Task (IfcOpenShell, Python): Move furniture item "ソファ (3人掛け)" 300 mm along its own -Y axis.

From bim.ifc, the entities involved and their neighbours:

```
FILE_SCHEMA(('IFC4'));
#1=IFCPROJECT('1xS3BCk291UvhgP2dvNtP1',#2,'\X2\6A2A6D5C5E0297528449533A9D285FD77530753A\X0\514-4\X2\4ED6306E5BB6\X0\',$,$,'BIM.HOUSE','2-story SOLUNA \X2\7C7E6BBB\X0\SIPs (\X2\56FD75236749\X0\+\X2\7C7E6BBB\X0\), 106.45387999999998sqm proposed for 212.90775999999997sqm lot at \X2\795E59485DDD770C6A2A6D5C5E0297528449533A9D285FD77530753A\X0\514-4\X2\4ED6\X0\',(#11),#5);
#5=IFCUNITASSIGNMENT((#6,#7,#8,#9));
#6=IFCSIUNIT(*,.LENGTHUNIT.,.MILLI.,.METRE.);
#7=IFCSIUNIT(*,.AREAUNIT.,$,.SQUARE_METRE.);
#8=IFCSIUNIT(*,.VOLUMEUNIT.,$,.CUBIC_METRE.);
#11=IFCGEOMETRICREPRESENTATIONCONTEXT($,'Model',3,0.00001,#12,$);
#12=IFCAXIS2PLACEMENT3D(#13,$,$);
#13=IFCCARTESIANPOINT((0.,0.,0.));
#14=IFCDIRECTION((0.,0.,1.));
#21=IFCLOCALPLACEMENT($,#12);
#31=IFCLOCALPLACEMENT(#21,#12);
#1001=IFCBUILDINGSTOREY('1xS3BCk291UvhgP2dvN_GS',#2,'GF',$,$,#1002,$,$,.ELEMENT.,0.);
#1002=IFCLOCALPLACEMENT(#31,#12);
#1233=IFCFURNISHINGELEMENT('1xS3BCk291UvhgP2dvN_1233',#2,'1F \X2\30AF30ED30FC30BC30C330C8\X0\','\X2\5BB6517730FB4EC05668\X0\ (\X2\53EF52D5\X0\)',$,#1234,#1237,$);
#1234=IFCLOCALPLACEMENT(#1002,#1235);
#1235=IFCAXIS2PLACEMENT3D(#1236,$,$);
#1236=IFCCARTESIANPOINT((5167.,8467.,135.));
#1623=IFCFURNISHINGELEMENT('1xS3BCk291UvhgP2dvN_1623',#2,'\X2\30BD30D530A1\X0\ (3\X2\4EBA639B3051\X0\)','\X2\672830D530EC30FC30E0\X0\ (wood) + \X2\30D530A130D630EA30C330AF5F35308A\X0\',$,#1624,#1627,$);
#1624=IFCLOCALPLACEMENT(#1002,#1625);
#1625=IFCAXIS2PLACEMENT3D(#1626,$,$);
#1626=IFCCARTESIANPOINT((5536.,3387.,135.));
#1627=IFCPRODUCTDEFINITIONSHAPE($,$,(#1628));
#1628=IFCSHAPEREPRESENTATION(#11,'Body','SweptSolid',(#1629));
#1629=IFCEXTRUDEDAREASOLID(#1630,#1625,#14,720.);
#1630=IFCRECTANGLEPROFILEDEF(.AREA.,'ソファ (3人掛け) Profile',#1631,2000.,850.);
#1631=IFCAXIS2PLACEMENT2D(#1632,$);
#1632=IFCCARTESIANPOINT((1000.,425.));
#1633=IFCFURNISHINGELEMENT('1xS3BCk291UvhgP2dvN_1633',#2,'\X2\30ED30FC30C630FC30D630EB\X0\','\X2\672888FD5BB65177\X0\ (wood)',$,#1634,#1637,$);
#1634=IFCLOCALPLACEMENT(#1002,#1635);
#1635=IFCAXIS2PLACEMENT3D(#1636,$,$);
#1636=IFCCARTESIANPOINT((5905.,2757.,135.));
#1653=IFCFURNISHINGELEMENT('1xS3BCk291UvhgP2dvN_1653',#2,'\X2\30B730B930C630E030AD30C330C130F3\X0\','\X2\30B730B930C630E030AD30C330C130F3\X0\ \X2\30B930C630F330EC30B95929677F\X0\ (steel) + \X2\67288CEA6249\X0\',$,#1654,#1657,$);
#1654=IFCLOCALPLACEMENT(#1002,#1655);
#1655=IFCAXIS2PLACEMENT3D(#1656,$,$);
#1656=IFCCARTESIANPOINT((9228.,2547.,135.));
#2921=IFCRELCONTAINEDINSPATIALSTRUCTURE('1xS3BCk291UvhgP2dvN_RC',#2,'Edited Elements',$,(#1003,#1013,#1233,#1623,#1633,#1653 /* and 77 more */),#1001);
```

```python
import ifcopenshell
import ifcopenshell.api.geometry
import ifcopenshell.util.placement
import ifcopenshell.util.unit

model = ifcopenshell.open("bim.ifc")
unit_scale = ifcopenshell.util.unit.calculate_unit_scale(model)

item = model.by_guid("1xS3BCk291UvhgP2dvN_1623")
matrix = ifcopenshell.util.placement.get_local_placement(item.ObjectPlacement)
matrix[:3, 3] -= matrix[:3, 1] * 0.3 / unit_scale
ifcopenshell.api.geometry.edit_object_placement(model, product=item, matrix=matrix, is_si=False)

print(ifcopenshell.util.placement.get_local_placement(item.ObjectPlacement).round(3) + 0.0)

model.write("bim_updated.ifc")
```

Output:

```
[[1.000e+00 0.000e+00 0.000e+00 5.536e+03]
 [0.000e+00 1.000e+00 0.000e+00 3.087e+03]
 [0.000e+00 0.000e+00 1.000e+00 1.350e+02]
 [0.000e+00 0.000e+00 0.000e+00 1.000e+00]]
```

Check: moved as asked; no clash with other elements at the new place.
